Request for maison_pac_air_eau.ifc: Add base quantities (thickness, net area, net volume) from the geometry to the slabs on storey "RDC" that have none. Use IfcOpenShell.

First a look at what the model holds.

```python
import ifcopenshell
import ifcopenshell.util.element
import ifcopenshell.util.unit

model = ifcopenshell.open("maison_pac_air_eau.ifc")
print(model.schema)
for unit_type in ("LENGTHUNIT", "AREAUNIT", "VOLUMEUNIT"):
    print(unit_type, ifcopenshell.util.unit.calculate_unit_scale(model, unit_type))
storey = next(s for s in model.by_type("IfcBuildingStorey") if s.Name == "RDC")
slabs = [e for e in ifcopenshell.util.element.get_decomposition(storey) if e.is_a("IfcSlab")]
for e in sorted(slabs, key=lambda e: e.id()):
    print(e.id(), e.is_a(), e.Name, list(ifcopenshell.util.element.get_psets(e, qtos_only=True)), sep=" | ")
```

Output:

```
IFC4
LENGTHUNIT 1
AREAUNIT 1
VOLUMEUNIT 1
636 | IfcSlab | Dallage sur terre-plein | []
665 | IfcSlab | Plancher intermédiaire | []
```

```python
import ifcopenshell
import ifcopenshell.api.pset
import ifcopenshell.geom
import ifcopenshell.util.element
import ifcopenshell.util.shape
import ifcopenshell.util.unit

model = ifcopenshell.open("maison_pac_air_eau.ifc")
unit_scale = ifcopenshell.util.unit.calculate_unit_scale(model)
area_scale = ifcopenshell.util.unit.calculate_unit_scale(model, "AREAUNIT")
volume_scale = ifcopenshell.util.unit.calculate_unit_scale(model, "VOLUMEUNIT")
settings = ifcopenshell.geom.settings()

storey = next(s for s in model.by_type("IfcBuildingStorey") if s.Name == "RDC")
slabs = [e for e in ifcopenshell.util.element.get_decomposition(storey) if e.is_a("IfcSlab")]

for e in sorted(slabs, key=lambda e: e.id()):
    if ifcopenshell.util.element.get_psets(e, qtos_only=True, should_inherit=False):
        continue
    # Geometry comes back in metres, in the element's own axes.
    shape = ifcopenshell.geom.create_shape(settings, e)
    values = {
        "Width": ifcopenshell.util.shape.get_z(shape.geometry) / unit_scale,
        "NetArea": ifcopenshell.util.shape.get_footprint_area(shape.geometry) / area_scale,
        "NetVolume": ifcopenshell.util.shape.get_volume(shape.geometry) / volume_scale,
    }
    qto = ifcopenshell.api.pset.add_qto(model, product=e, name="Qto_SlabBaseQuantities")
    ifcopenshell.api.pset.edit_qto(model, qto=qto, properties=values)
    print(e.id(), {k: round(v, 3) for k, v in values.items()})

model.write("maison_pac_air_eau-out.ifc")
```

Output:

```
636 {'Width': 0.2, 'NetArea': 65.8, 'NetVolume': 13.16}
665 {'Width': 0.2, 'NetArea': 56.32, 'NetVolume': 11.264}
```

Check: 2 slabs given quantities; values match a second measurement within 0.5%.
